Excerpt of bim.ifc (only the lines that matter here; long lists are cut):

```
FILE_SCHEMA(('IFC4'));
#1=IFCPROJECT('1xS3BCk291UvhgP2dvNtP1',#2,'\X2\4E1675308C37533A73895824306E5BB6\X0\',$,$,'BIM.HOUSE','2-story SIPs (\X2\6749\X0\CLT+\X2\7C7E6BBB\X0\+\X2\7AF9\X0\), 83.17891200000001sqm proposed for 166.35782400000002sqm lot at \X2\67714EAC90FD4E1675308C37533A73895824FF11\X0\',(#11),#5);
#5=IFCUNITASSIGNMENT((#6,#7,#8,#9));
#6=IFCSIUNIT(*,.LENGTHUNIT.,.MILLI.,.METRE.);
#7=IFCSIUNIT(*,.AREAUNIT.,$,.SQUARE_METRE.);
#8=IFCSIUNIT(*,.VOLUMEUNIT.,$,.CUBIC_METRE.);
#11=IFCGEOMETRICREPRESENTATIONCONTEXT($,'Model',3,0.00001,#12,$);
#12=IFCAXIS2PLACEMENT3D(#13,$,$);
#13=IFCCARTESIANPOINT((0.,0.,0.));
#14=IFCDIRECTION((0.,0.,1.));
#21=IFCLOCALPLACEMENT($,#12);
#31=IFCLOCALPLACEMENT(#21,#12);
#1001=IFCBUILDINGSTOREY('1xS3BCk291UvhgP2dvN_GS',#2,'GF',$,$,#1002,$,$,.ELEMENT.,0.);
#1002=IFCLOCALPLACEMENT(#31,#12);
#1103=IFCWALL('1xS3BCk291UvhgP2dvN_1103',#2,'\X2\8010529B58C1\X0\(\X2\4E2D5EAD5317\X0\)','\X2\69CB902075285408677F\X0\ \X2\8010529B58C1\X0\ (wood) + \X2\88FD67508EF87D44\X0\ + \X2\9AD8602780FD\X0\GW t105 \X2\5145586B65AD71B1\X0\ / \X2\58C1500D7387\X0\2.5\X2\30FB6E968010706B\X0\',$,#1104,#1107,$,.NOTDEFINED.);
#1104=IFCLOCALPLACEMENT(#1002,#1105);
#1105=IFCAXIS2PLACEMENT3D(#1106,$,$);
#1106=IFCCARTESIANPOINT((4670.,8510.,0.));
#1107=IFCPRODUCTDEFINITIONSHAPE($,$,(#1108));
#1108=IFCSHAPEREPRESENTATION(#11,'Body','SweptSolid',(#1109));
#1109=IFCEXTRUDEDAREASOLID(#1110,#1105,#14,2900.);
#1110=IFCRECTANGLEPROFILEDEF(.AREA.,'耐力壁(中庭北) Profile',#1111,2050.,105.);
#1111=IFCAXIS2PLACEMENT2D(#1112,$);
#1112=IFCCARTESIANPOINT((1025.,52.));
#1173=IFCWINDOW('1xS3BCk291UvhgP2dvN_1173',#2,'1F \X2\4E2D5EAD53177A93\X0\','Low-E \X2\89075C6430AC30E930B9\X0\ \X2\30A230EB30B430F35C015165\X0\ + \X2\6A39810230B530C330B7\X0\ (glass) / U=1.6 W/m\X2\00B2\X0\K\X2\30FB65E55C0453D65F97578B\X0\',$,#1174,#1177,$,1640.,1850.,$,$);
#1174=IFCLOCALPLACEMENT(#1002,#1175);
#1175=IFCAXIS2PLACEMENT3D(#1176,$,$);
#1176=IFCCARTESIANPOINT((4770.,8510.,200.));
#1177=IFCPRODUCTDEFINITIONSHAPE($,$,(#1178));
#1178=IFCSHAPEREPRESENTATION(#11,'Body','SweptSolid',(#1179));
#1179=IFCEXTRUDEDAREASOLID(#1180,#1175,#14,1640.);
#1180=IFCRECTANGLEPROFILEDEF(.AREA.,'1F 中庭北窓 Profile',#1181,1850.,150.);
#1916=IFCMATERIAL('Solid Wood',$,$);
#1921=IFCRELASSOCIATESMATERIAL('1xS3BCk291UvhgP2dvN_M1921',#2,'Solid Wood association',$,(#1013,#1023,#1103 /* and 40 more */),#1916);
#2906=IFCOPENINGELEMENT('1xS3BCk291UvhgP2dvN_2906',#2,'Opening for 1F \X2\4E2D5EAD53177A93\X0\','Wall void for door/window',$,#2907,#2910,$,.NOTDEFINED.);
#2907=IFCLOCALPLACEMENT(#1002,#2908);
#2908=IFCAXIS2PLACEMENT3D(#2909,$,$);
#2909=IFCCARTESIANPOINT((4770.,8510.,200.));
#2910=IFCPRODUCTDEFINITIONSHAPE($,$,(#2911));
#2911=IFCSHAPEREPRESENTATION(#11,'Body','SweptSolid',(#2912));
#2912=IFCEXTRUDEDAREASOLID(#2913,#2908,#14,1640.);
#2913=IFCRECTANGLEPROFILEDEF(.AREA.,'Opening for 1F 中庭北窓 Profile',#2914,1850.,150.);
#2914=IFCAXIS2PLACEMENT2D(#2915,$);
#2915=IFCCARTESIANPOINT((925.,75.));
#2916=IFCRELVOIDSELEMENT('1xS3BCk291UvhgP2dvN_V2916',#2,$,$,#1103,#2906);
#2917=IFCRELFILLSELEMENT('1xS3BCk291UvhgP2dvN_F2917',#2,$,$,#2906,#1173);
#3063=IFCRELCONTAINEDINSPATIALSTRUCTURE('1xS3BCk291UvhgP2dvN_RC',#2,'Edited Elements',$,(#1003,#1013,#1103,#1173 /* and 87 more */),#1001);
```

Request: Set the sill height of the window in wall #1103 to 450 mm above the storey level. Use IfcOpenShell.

```python
import numpy as np
import ifcopenshell
import ifcopenshell.api.geometry
import ifcopenshell.geom
import ifcopenshell.util.element
import ifcopenshell.util.placement
import ifcopenshell.util.shape
import ifcopenshell.util.unit

model = ifcopenshell.open("bim.ifc")
unit_scale = ifcopenshell.util.unit.calculate_unit_scale(model)

window = model.by_guid("1xS3BCk291UvhgP2dvN_1173")
opening = window.FillsVoids[0].RelatingOpeningElement
storey = ifcopenshell.util.element.get_container(window, ifc_class="IfcBuildingStorey")
level = ifcopenshell.util.placement.get_local_placement(storey.ObjectPlacement)[2, 3]

# The opening's origin need not be at the sill, so measure its lowest point.
shape = ifcopenshell.geom.create_shape(ifcopenshell.geom.settings(), opening)
bottom = ifcopenshell.util.shape.get_shape_bottom_elevation(shape, shape.geometry) / unit_scale
dz = level + 0.45 / unit_scale - bottom

shift = np.array([0.0, 0.0, dz])
# The window is not placed relative to its opening, so move both.
for product in (opening, window):
    matrix = ifcopenshell.util.placement.get_local_placement(product.ObjectPlacement)
    matrix[:3, 3] += shift
    ifcopenshell.api.geometry.edit_object_placement(model, product=product, matrix=matrix, is_si=False)

print(f"moved by {dz * unit_scale:+.3f} m")

model.write("bim_edited.ifc")
```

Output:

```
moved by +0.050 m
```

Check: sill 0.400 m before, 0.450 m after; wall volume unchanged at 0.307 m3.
